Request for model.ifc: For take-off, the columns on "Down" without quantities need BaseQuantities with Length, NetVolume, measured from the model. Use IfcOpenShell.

First a look at what the model holds.

```python
import ifcopenshell
import ifcopenshell.util.element
import ifcopenshell.util.unit

model = ifcopenshell.open("model.ifc")
print(model.schema)
for unit_type in ("LENGTHUNIT", "AREAUNIT", "VOLUMEUNIT"):
    print(unit_type, ifcopenshell.util.unit.calculate_unit_scale(model, unit_type))
storey = next(s for s in model.by_type("IfcBuildingStorey") if s.Name == "Down")
columns = [e for e in ifcopenshell.util.element.get_decomposition(storey) if e.is_a("IfcColumn")]
for e in sorted(columns, key=lambda e: e.id()):
    print(e.id(), e.is_a(), e.Name, list(ifcopenshell.util.element.get_psets(e, qtos_only=True)), sep=" | ")
```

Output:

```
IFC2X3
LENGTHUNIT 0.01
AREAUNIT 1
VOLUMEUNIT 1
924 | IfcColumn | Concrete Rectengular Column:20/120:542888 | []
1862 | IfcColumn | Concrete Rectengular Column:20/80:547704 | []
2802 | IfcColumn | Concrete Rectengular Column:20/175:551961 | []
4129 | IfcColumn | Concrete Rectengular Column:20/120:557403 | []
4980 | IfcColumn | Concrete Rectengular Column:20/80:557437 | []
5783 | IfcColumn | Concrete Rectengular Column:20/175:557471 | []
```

```python
import ifcopenshell
import ifcopenshell.api.pset
import ifcopenshell.geom
import ifcopenshell.util.element
import ifcopenshell.util.shape
import ifcopenshell.util.unit

model = ifcopenshell.open("model.ifc")
unit_scale = ifcopenshell.util.unit.calculate_unit_scale(model)
volume_scale = ifcopenshell.util.unit.calculate_unit_scale(model, "VOLUMEUNIT")
settings = ifcopenshell.geom.settings()

storey = next(s for s in model.by_type("IfcBuildingStorey") if s.Name == "Down")
columns = [e for e in ifcopenshell.util.element.get_decomposition(storey) if e.is_a("IfcColumn")]

for e in sorted(columns, key=lambda e: e.id()):
    if ifcopenshell.util.element.get_psets(e, qtos_only=True, should_inherit=False):
        continue
    # Geometry comes back in metres, in the element's own axes.
    shape = ifcopenshell.geom.create_shape(settings, e)
    values = {
        "Length": ifcopenshell.util.shape.get_z(shape.geometry) / unit_scale,
        "NetVolume": ifcopenshell.util.shape.get_volume(shape.geometry) / volume_scale,
    }
    qto = ifcopenshell.api.pset.add_qto(model, product=e, name="BaseQuantities")
    ifcopenshell.api.pset.edit_qto(model, qto=qto, properties=values)
    print(e.id(), {k: round(v, 3) for k, v in values.items()})

model.write("model_v2.ifc")
```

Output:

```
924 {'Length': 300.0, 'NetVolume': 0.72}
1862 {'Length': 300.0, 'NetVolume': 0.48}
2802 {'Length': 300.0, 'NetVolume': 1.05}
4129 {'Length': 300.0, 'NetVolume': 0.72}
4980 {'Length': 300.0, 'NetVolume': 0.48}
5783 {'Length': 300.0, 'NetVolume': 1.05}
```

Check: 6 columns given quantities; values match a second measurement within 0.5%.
